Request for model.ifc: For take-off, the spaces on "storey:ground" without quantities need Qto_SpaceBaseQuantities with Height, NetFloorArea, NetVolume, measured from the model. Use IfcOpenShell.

First a look at what the model holds.

```python
import ifcopenshell
import ifcopenshell.util.element
import ifcopenshell.util.unit

model = ifcopenshell.open("model.ifc")
print(model.schema)
for unit_type in ("LENGTHUNIT", "AREAUNIT", "VOLUMEUNIT"):
    print(unit_type, ifcopenshell.util.unit.calculate_unit_scale(model, unit_type))
storey = next(s for s in model.by_type("IfcBuildingStorey") if s.Name == "storey:ground")
spaces = [e for e in ifcopenshell.util.element.get_decomposition(storey) if e.is_a("IfcSpace")]
for e in sorted(spaces, key=lambda e: e.id()):
    print(e.id(), e.is_a(), e.Name, list(ifcopenshell.util.element.get_psets(e, qtos_only=True)), sep=" | ")
```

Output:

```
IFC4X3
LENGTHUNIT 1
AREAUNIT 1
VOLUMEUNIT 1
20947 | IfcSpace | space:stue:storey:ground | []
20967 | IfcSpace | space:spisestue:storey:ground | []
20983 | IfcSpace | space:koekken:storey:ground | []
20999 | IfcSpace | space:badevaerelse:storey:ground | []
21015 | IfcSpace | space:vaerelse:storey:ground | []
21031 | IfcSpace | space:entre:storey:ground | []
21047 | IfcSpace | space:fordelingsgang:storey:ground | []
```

```python
import ifcopenshell
import ifcopenshell.api.pset
import ifcopenshell.geom
import ifcopenshell.util.element
import ifcopenshell.util.shape
import ifcopenshell.util.unit

model = ifcopenshell.open("model.ifc")
unit_scale = ifcopenshell.util.unit.calculate_unit_scale(model)
area_scale = ifcopenshell.util.unit.calculate_unit_scale(model, "AREAUNIT")
volume_scale = ifcopenshell.util.unit.calculate_unit_scale(model, "VOLUMEUNIT")
settings = ifcopenshell.geom.settings()

storey = next(s for s in model.by_type("IfcBuildingStorey") if s.Name == "storey:ground")
spaces = [e for e in ifcopenshell.util.element.get_decomposition(storey) if e.is_a("IfcSpace")]

for e in sorted(spaces, key=lambda e: e.id()):
    if ifcopenshell.util.element.get_psets(e, qtos_only=True, should_inherit=False):
        continue
    # Geometry comes back in metres, in the element's own axes.
    shape = ifcopenshell.geom.create_shape(settings, e)
    values = {
        "Height": ifcopenshell.util.shape.get_z(shape.geometry) / unit_scale,
        "NetFloorArea": ifcopenshell.util.shape.get_footprint_area(shape.geometry) / area_scale,
        "NetVolume": ifcopenshell.util.shape.get_volume(shape.geometry) / volume_scale,
    }
    qto = ifcopenshell.api.pset.add_qto(model, product=e, name="Qto_SpaceBaseQuantities")
    ifcopenshell.api.pset.edit_qto(model, qto=qto, properties=values)
    print(e.id(), {k: round(v, 3) for k, v in values.items()})

model.write("model_rev.ifc")
```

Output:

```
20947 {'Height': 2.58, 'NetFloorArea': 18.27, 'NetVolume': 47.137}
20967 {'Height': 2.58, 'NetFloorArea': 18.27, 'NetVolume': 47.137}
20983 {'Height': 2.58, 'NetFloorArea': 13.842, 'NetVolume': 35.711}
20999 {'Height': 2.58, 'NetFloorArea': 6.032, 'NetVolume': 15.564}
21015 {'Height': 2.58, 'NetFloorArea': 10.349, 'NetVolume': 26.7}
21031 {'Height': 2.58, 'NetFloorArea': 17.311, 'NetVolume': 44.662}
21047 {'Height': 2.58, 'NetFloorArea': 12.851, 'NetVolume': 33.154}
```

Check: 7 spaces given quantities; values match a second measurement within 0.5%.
